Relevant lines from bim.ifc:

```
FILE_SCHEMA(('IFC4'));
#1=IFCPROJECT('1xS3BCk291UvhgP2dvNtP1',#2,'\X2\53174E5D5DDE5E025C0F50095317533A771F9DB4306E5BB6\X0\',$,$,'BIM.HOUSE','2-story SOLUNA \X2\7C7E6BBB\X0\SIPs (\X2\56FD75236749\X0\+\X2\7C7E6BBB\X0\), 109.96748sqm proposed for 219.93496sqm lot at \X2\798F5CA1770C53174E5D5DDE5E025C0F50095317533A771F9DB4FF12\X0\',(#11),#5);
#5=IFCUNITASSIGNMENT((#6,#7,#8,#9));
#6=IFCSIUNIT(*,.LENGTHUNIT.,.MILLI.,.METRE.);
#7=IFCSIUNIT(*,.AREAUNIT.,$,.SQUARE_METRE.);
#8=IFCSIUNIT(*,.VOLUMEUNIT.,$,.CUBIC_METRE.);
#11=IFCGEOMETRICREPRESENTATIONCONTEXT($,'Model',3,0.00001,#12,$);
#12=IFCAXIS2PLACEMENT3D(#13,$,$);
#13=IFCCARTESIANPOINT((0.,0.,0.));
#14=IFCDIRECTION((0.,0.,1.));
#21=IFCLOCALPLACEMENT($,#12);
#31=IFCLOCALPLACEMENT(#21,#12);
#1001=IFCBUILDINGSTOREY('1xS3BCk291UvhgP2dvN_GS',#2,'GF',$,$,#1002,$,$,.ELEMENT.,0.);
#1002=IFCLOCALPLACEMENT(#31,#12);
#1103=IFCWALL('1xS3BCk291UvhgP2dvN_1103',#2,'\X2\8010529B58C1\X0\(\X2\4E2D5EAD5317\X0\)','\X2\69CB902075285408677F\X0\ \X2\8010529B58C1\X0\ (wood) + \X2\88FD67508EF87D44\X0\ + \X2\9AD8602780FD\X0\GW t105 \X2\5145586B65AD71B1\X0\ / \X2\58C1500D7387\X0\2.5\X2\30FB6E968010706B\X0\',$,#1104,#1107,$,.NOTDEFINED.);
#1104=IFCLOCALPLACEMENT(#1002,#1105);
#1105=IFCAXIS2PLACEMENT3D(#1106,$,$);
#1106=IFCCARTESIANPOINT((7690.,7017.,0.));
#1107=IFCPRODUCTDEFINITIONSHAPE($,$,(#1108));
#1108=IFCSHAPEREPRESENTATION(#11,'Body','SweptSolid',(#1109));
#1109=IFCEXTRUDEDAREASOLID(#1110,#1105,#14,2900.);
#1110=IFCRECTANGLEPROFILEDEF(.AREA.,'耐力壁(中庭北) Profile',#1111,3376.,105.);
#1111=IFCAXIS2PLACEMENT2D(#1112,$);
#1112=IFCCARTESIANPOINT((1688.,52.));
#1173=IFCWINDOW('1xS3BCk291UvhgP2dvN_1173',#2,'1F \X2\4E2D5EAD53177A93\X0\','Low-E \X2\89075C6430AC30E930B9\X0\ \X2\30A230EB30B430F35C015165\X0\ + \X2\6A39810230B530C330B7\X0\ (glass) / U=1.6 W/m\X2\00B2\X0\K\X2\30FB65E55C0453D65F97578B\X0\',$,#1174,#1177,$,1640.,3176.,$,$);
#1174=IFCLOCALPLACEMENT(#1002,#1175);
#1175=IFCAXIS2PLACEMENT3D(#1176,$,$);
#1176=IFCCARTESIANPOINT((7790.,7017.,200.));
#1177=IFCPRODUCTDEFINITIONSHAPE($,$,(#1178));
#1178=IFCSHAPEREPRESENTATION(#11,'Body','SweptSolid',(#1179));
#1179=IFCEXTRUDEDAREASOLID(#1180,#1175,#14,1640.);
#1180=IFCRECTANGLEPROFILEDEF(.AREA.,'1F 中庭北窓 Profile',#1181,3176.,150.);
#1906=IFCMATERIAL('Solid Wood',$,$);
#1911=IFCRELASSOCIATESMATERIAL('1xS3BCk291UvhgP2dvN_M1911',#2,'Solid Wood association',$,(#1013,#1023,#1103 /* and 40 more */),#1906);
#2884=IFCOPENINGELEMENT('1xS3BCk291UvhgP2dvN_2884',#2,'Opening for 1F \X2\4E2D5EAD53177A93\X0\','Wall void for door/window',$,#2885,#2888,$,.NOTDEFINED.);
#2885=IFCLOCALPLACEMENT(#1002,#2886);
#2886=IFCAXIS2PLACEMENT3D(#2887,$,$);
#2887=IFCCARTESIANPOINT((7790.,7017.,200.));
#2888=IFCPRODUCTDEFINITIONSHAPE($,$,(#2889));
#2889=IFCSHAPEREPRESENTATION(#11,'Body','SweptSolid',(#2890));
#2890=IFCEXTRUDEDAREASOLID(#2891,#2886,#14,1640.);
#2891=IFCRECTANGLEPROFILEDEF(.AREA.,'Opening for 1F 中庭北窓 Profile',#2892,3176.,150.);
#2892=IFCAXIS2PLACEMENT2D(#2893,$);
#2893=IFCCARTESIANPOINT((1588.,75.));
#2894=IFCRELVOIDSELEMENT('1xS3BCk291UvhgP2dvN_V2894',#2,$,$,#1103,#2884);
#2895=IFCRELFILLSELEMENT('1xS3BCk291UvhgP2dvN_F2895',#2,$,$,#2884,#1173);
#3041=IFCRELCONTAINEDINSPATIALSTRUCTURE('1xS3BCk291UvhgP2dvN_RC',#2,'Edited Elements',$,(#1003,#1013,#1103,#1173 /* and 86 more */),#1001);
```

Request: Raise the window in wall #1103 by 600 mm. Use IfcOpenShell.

```python
import numpy as np
import ifcopenshell
import ifcopenshell.api.geometry
import ifcopenshell.util.placement
import ifcopenshell.util.unit

model = ifcopenshell.open("bim.ifc")
unit_scale = ifcopenshell.util.unit.calculate_unit_scale(model)

window = model.by_guid("1xS3BCk291UvhgP2dvN_1173")
opening = window.FillsVoids[0].RelatingOpeningElement
dz = 600.0

shift = np.array([0.0, 0.0, dz])
# The window is not placed relative to its opening, so move both.
for product in (opening, window):
    matrix = ifcopenshell.util.placement.get_local_placement(product.ObjectPlacement)
    matrix[:3, 3] += shift
    ifcopenshell.api.geometry.edit_object_placement(model, product=product, matrix=matrix, is_si=False)

print(f"moved by {dz * unit_scale:+.3f} m")

model.write("bim_v2.ifc")
```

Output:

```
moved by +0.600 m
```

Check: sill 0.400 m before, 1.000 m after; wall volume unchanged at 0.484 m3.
